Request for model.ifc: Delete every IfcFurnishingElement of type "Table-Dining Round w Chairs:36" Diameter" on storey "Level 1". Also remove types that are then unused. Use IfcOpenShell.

First a look at what the model holds.

```python
import ifcopenshell
import ifcopenshell.util.element

model = ifcopenshell.open("model.ifc")
print(model.schema)
storey = next(s for s in model.by_type("IfcBuildingStorey") if s.Name == "Level 1")
furniture = [e for e in ifcopenshell.util.element.get_decomposition(storey) if e.is_a("IfcFurnishingElement")]
seen = {}
for e in furniture:
    element_type = ifcopenshell.util.element.get_type(e)
    name = element_type.Name if element_type not in (None, e) else None
    seen[name] = seen.get(name, 0) + 1
for name, count in sorted(seen.items(), key=str):
    print(count, "x", name)
```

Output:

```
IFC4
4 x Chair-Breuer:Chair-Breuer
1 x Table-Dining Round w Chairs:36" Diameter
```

```python
import ifcopenshell
import ifcopenshell.api.root
import ifcopenshell.util.element

model = ifcopenshell.open("model.ifc")

storey = next(s for s in model.by_type("IfcBuildingStorey") if s.Name == "Level 1")
furniture = [e for e in ifcopenshell.util.element.get_decomposition(storey) if e.is_a("IfcFurnishingElement")]
targets = [e for e in furniture if (t := ifcopenshell.util.element.get_type(e)) not in (None, e) and t.Name == 'Table-Dining Round w Chairs:36" Diameter']
types = {ifcopenshell.util.element.get_type(e) for e in targets} - {None, *targets}

for e in targets:
    ifcopenshell.api.root.remove_product(model, product=e)
print(len(targets), "removed")

unused = [t for t in types if not ifcopenshell.util.element.get_types(t)]
for t in unused:
    ifcopenshell.api.root.remove_product(model, product=t)
print(len(unused), "unused types removed")

model.write("model_edited.ifc")
```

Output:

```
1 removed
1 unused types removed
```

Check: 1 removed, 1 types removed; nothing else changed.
